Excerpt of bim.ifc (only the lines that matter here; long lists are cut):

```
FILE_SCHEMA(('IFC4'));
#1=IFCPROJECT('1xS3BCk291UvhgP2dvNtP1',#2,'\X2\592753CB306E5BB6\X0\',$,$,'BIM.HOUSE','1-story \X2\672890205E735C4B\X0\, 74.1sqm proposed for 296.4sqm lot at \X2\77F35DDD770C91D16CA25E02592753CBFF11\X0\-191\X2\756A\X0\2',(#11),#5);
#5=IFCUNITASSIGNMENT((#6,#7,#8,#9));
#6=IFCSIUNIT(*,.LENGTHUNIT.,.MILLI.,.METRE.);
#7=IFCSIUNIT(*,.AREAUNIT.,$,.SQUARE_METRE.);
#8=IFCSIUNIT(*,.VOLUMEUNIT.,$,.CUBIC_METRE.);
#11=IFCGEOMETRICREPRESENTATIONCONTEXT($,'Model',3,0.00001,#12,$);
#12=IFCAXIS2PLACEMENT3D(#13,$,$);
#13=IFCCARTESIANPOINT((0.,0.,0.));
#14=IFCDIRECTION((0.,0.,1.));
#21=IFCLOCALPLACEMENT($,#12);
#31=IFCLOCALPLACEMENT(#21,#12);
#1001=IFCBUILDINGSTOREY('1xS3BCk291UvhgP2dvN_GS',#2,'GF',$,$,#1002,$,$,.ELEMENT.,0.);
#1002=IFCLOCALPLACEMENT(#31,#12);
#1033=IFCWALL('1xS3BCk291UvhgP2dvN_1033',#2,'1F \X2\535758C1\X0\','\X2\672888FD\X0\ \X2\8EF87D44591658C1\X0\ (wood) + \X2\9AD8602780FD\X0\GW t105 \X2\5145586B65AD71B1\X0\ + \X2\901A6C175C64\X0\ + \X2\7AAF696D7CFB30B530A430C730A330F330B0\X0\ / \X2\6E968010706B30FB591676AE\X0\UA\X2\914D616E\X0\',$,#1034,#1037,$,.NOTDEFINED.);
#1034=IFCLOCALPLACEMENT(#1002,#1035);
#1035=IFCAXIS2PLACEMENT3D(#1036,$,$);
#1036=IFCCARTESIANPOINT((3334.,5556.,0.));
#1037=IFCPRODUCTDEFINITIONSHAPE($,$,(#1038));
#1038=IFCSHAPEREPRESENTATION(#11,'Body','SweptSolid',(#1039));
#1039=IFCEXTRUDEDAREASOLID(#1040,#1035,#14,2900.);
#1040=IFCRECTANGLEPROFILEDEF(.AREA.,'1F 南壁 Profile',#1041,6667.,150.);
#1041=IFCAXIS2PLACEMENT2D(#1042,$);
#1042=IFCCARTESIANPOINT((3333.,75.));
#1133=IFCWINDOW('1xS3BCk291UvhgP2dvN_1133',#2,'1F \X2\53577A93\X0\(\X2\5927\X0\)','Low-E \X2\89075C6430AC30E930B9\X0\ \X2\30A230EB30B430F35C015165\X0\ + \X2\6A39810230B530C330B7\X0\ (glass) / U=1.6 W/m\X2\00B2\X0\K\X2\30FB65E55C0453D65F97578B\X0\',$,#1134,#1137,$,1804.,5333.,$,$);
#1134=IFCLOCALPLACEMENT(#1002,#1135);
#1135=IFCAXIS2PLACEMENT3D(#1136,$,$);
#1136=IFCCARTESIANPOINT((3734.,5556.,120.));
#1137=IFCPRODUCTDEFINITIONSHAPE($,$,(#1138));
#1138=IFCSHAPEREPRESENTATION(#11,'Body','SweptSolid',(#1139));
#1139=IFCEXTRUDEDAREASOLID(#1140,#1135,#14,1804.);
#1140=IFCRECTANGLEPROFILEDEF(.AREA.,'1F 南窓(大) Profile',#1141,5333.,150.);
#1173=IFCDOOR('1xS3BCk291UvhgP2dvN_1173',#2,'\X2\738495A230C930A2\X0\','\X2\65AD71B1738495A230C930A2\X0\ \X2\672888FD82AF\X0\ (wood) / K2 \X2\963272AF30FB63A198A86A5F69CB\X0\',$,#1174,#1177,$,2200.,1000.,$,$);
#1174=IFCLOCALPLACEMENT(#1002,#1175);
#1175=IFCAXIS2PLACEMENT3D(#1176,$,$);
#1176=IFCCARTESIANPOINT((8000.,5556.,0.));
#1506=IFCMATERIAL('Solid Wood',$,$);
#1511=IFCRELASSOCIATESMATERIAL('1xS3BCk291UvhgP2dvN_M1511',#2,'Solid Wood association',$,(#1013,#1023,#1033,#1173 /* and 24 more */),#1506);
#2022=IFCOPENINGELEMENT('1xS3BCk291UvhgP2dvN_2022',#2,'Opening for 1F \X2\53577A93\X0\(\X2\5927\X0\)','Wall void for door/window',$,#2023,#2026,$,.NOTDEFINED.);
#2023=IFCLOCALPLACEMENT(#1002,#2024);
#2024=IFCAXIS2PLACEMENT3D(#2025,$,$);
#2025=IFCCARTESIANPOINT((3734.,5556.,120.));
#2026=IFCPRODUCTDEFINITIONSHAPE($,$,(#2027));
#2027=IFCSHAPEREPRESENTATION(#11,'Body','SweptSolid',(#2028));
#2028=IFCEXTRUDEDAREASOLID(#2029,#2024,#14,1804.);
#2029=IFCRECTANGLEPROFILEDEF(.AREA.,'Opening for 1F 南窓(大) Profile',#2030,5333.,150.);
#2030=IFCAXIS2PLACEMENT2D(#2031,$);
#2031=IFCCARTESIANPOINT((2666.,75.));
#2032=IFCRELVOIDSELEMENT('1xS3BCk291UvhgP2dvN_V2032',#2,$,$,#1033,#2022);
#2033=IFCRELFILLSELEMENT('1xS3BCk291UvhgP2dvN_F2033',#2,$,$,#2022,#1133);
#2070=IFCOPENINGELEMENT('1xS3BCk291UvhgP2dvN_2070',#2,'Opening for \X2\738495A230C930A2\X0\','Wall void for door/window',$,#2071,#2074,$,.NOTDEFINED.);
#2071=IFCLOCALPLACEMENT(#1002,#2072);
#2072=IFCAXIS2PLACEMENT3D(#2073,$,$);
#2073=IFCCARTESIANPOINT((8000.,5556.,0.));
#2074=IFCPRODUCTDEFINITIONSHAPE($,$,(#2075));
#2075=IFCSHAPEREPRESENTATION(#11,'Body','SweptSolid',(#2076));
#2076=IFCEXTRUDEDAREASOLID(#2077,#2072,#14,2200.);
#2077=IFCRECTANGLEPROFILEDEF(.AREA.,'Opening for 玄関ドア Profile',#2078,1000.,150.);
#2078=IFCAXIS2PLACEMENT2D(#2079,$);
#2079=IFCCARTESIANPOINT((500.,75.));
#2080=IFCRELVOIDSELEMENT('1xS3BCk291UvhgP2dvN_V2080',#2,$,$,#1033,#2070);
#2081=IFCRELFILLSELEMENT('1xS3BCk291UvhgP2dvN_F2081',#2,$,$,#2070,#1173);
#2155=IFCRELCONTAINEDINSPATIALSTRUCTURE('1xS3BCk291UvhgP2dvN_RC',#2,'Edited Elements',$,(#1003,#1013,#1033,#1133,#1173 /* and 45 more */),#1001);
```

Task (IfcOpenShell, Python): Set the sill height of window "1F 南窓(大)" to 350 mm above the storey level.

```python
import numpy as np
import ifcopenshell
import ifcopenshell.api.geometry
import ifcopenshell.geom
import ifcopenshell.util.element
import ifcopenshell.util.placement
import ifcopenshell.util.shape
import ifcopenshell.util.unit

model = ifcopenshell.open("bim.ifc")
unit_scale = ifcopenshell.util.unit.calculate_unit_scale(model)

window = model.by_guid("1xS3BCk291UvhgP2dvN_1133")
opening = window.FillsVoids[0].RelatingOpeningElement
storey = ifcopenshell.util.element.get_container(window, ifc_class="IfcBuildingStorey")
level = ifcopenshell.util.placement.get_local_placement(storey.ObjectPlacement)[2, 3]

# The opening's origin need not be at the sill, so measure its lowest point.
shape = ifcopenshell.geom.create_shape(ifcopenshell.geom.settings(), opening)
bottom = ifcopenshell.util.shape.get_shape_bottom_elevation(shape, shape.geometry) / unit_scale
dz = level + 0.35 / unit_scale - bottom

shift = np.array([0.0, 0.0, dz])
# The window is not placed relative to its opening, so move both.
for product in (opening, window):
    matrix = ifcopenshell.util.placement.get_local_placement(product.ObjectPlacement)
    matrix[:3, 3] += shift
    ifcopenshell.api.geometry.edit_object_placement(model, product=product, matrix=matrix, is_si=False)

print(f"moved by {dz * unit_scale:+.3f} m")

model.write("bim_v2.ifc")
```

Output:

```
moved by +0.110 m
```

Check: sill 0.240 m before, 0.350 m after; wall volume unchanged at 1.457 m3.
